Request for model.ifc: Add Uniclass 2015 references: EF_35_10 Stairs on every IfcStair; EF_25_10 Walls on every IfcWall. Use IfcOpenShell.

First a look at what the model holds.

```python
import ifcopenshell

model = ifcopenshell.open("model.ifc")
print(model.schema)
print("classifications:", [c.Name for c in model.by_type("IfcClassification")])
for ifc_class in ("IfcDoor", "IfcRoof", "IfcStair", "IfcWall", "IfcWindow"):
    print(ifc_class, len(model.by_type(ifc_class)))
```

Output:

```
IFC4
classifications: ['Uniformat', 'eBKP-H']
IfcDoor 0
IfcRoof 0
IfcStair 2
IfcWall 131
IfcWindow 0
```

```python
import ifcopenshell
import ifcopenshell.api.classification

model = ifcopenshell.open("model.ifc")

system = ifcopenshell.api.classification.add_classification(model, classification="Uniclass 2015")

codes = {
    "IfcStair": ("EF_35_10", "Stairs"),
    "IfcWall": ("EF_25_10", "Walls"),
}
for ifc_class, (code, name) in codes.items():
    products = model.by_type(ifc_class)
    ifcopenshell.api.classification.add_reference(
        model, products=products, classification=system, identification=code, name=name
    )
    print(code, len(products))

model.write("model_v2.ifc")
```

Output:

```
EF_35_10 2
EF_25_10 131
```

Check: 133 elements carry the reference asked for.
